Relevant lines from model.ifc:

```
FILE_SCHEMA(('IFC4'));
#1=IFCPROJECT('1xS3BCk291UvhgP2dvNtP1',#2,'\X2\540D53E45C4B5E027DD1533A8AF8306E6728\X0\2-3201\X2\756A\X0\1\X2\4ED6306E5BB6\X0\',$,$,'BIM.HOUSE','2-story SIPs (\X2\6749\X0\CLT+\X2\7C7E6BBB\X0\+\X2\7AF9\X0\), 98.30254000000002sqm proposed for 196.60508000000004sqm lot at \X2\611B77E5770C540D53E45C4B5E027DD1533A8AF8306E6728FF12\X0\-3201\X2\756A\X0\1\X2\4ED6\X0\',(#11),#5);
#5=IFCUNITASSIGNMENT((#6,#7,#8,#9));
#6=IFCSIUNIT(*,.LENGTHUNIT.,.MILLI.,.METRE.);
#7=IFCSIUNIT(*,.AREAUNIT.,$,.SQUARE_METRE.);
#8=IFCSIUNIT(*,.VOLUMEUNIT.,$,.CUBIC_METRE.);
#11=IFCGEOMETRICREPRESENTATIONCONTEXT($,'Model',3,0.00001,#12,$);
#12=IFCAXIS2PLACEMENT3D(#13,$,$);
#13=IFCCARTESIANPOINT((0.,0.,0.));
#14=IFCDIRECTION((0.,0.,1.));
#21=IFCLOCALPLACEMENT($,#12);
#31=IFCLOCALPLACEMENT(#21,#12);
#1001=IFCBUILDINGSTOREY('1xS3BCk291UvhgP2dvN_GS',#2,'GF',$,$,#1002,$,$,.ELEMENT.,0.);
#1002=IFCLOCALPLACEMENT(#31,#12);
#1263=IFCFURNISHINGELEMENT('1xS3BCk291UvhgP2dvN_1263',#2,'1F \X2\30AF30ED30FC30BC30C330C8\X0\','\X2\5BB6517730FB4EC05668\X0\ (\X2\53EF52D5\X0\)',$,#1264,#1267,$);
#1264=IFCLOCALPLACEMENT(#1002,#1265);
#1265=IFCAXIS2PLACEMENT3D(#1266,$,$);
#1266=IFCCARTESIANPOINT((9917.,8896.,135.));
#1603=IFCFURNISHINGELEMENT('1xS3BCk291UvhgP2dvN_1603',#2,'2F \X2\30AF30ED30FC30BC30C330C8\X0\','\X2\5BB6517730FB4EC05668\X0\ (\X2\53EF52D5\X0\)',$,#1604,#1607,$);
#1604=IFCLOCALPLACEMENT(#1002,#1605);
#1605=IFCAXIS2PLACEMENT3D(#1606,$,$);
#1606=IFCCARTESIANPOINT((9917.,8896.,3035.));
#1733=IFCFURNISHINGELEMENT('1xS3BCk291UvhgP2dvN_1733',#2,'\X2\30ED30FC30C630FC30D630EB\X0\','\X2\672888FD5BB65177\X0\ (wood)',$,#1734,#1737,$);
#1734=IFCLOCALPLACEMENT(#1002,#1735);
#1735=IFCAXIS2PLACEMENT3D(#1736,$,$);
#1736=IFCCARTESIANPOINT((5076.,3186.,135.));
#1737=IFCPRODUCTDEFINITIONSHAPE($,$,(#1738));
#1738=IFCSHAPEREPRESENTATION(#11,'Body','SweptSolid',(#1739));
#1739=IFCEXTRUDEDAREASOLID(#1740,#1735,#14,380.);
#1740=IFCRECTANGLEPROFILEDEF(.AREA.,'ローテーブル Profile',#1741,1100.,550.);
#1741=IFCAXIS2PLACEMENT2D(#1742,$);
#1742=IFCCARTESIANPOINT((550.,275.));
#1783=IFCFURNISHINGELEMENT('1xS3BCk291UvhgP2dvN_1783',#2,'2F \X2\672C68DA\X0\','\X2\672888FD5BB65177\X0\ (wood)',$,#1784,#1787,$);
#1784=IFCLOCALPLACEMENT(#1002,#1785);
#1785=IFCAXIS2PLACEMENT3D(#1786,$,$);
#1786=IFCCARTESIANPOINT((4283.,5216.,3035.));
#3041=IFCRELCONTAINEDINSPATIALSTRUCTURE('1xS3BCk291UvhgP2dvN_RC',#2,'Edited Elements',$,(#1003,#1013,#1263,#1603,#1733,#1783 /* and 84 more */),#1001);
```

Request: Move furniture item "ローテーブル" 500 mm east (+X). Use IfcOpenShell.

```python
import ifcopenshell
import ifcopenshell.api.geometry
import ifcopenshell.util.placement

model = ifcopenshell.open("model.ifc")

item = model.by_id(1733)
matrix = ifcopenshell.util.placement.get_local_placement(item.ObjectPlacement)
matrix[0, 3] += 500.0
ifcopenshell.api.geometry.edit_object_placement(model, product=item, matrix=matrix, is_si=False)

print(ifcopenshell.util.placement.get_local_placement(item.ObjectPlacement).round(3) + 0.0)

model.write("model_rev.ifc")
```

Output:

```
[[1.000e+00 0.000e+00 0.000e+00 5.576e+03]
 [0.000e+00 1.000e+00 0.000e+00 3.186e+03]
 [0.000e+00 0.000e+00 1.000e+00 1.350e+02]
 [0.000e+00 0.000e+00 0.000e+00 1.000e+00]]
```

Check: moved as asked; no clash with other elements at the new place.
